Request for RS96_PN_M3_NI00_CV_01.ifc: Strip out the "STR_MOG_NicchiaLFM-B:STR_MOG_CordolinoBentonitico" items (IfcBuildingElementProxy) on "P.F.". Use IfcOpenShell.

First a look at what the model holds.

```python
import ifcopenshell
import ifcopenshell.util.element

model = ifcopenshell.open("RS96_PN_M3_NI00_CV_01.ifc")
print(model.schema)
storey = next(s for s in model.by_type("IfcBuildingStorey") if s.Name == "P.F.")
proxies = [e for e in ifcopenshell.util.element.get_decomposition(storey) if e.is_a("IfcBuildingElementProxy")]
seen = {}
for e in proxies:
    element_type = ifcopenshell.util.element.get_type(e)
    name = element_type.Name if element_type not in (None, e) else None
    seen[name] = seen.get(name, 0) + 1
for name, count in sorted(seen.items(), key=str):
    print(count, "x", name)
```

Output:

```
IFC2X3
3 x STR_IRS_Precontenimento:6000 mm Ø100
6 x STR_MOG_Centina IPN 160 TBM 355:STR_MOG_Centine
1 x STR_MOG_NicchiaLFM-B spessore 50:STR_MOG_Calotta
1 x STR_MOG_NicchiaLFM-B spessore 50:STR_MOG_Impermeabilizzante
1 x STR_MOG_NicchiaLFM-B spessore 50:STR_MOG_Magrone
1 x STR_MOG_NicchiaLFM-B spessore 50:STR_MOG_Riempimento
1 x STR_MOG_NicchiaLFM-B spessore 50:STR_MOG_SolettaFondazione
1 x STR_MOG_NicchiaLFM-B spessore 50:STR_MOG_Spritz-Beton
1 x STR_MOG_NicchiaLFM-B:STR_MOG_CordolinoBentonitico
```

```python
import ifcopenshell
import ifcopenshell.api.root
import ifcopenshell.util.element

model = ifcopenshell.open("RS96_PN_M3_NI00_CV_01.ifc")

storey = next(s for s in model.by_type("IfcBuildingStorey") if s.Name == "P.F.")
proxies = [e for e in ifcopenshell.util.element.get_decomposition(storey) if e.is_a("IfcBuildingElementProxy")]
targets = [e for e in proxies if (t := ifcopenshell.util.element.get_type(e)) not in (None, e) and t.Name == "STR_MOG_NicchiaLFM-B:STR_MOG_CordolinoBentonitico"]

for e in targets:
    ifcopenshell.api.root.remove_product(model, product=e)
print(len(targets), "removed")

model.write("RS96_PN_M3_NI00_CV_01_updated.ifc")
```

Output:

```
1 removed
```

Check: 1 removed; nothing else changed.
